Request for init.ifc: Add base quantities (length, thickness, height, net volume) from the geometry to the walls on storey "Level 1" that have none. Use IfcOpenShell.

First a look at what the model holds.

```python
import ifcopenshell
import ifcopenshell.util.element
import ifcopenshell.util.unit

model = ifcopenshell.open("init.ifc")
print(model.schema)
for unit_type in ("LENGTHUNIT", "AREAUNIT", "VOLUMEUNIT"):
    print(unit_type, ifcopenshell.util.unit.calculate_unit_scale(model, unit_type))
storey = next(s for s in model.by_type("IfcBuildingStorey") if s.Name == "Level 1")
walls = [e for e in ifcopenshell.util.element.get_decomposition(storey) if e.is_a("IfcWall")]
for e in sorted(walls, key=lambda e: e.id()):
    print(e.id(), e.is_a(), e.Name, list(ifcopenshell.util.element.get_psets(e, qtos_only=True)), sep=" | ")
```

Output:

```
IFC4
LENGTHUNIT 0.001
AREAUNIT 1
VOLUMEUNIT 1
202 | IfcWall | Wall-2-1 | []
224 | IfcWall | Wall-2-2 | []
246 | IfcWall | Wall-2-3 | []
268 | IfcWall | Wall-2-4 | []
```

```python
import ifcopenshell
import ifcopenshell.api.pset
import ifcopenshell.geom
import ifcopenshell.util.element
import ifcopenshell.util.shape
import ifcopenshell.util.unit

model = ifcopenshell.open("init.ifc")
unit_scale = ifcopenshell.util.unit.calculate_unit_scale(model)
volume_scale = ifcopenshell.util.unit.calculate_unit_scale(model, "VOLUMEUNIT")
settings = ifcopenshell.geom.settings()

storey = next(s for s in model.by_type("IfcBuildingStorey") if s.Name == "Level 1")
walls = [e for e in ifcopenshell.util.element.get_decomposition(storey) if e.is_a("IfcWall")]

for e in sorted(walls, key=lambda e: e.id()):
    if ifcopenshell.util.element.get_psets(e, qtos_only=True, should_inherit=False):
        continue
    # Geometry comes back in metres, in the element's own axes.
    shape = ifcopenshell.geom.create_shape(settings, e)
    values = {
        "Length": ifcopenshell.util.shape.get_x(shape.geometry) / unit_scale,
        "Width": ifcopenshell.util.shape.get_y(shape.geometry) / unit_scale,
        "Height": ifcopenshell.util.shape.get_z(shape.geometry) / unit_scale,
        "NetVolume": ifcopenshell.util.shape.get_volume(shape.geometry) / volume_scale,
    }
    qto = ifcopenshell.api.pset.add_qto(model, product=e, name="Qto_WallBaseQuantities")
    ifcopenshell.api.pset.edit_qto(model, qto=qto, properties=values)
    print(e.id(), {k: round(v, 3) for k, v in values.items()})

model.write("init-out.ifc")
```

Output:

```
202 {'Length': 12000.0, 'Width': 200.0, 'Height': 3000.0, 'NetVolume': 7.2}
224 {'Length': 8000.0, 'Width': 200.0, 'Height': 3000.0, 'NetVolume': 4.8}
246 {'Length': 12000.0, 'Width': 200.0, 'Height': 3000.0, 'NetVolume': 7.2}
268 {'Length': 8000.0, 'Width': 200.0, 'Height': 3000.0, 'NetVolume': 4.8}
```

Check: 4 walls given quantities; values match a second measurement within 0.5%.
